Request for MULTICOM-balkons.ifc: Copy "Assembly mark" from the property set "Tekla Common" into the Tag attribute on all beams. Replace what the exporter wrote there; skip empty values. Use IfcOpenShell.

First a look at what the model holds.

```python
import ifcopenshell
import ifcopenshell.util.element

model = ifcopenshell.open("MULTICOM-balkons.ifc")
print(model.schema)
beams = model.by_type("IfcBeam")
print(len(beams), "beams")
for e in beams[:8]:
    source = ifcopenshell.util.element.get_pset(e, "Tekla Common", "Assembly mark")
    target = e.Tag
    print(e.id(), repr(source), repr(target), sep=" | ")
```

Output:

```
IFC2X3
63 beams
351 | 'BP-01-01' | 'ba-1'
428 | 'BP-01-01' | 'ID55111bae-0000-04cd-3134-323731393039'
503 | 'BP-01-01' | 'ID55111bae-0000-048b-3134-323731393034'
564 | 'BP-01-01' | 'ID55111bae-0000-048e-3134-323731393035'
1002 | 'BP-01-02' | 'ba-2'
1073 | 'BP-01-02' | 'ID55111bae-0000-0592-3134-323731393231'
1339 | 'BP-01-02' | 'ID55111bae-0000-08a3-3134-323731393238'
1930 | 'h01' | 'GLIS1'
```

```python
import ifcopenshell
import ifcopenshell.util.element

model = ifcopenshell.open("MULTICOM-balkons.ifc")

count = 0
for e in model.by_type("IfcBeam"):
    value = ifcopenshell.util.element.get_pset(e, "Tekla Common", "Assembly mark")
    current = e.Tag
    if not value or not value.strip() or current == value:
        continue
    e.Tag = value
    count += 1

print(count, "beams updated")

model.write("MULTICOM-balkons-out.ifc")
```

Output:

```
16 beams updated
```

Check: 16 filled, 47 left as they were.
